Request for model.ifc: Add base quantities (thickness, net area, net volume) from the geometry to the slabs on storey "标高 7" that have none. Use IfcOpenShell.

First a look at what the model holds.

```python
import ifcopenshell
import ifcopenshell.util.element
import ifcopenshell.util.unit

model = ifcopenshell.open("model.ifc")
print(model.schema)
for unit_type in ("LENGTHUNIT", "AREAUNIT", "VOLUMEUNIT"):
    print(unit_type, ifcopenshell.util.unit.calculate_unit_scale(model, unit_type))
storey = next(s for s in model.by_type("IfcBuildingStorey") if s.Name == "标高 7")
slabs = [e for e in ifcopenshell.util.element.get_decomposition(storey) if e.is_a("IfcSlab")]
for e in sorted(slabs, key=lambda e: e.id()):
    print(e.id(), e.is_a(), e.Name, list(ifcopenshell.util.element.get_psets(e, qtos_only=True)), sep=" | ")
```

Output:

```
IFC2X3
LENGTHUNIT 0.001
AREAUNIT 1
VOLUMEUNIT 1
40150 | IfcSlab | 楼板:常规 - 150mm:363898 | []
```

```python
import ifcopenshell
import ifcopenshell.api.pset
import ifcopenshell.geom
import ifcopenshell.util.element
import ifcopenshell.util.shape
import ifcopenshell.util.unit

model = ifcopenshell.open("model.ifc")
unit_scale = ifcopenshell.util.unit.calculate_unit_scale(model)
area_scale = ifcopenshell.util.unit.calculate_unit_scale(model, "AREAUNIT")
volume_scale = ifcopenshell.util.unit.calculate_unit_scale(model, "VOLUMEUNIT")
settings = ifcopenshell.geom.settings()

storey = next(s for s in model.by_type("IfcBuildingStorey") if s.Name == "标高 7")
slabs = [e for e in ifcopenshell.util.element.get_decomposition(storey) if e.is_a("IfcSlab")]

for e in sorted(slabs, key=lambda e: e.id()):
    if ifcopenshell.util.element.get_psets(e, qtos_only=True, should_inherit=False):
        continue
    # Geometry comes back in metres, in the element's own axes.
    shape = ifcopenshell.geom.create_shape(settings, e)
    values = {
        "Width": ifcopenshell.util.shape.get_z(shape.geometry) / unit_scale,
        "NetArea": ifcopenshell.util.shape.get_footprint_area(shape.geometry) / area_scale,
        "NetVolume": ifcopenshell.util.shape.get_volume(shape.geometry) / volume_scale,
    }
    qto = ifcopenshell.api.pset.add_qto(model, product=e, name="BaseQuantities")
    ifcopenshell.api.pset.edit_qto(model, qto=qto, properties=values)
    print(e.id(), {k: round(v, 3) for k, v in values.items()})

model.write("model_edited.ifc")
```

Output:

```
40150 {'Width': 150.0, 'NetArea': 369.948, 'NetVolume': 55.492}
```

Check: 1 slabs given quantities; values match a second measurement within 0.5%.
